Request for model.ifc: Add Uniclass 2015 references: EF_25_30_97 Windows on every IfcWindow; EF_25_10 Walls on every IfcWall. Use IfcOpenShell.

First a look at what the model holds.

```python
import ifcopenshell

model = ifcopenshell.open("model.ifc")
print(model.schema)
print("classifications:", [c.Name for c in model.by_type("IfcClassification")])
for ifc_class in ("IfcDoor", "IfcRoof", "IfcStair", "IfcWall", "IfcWindow"):
    print(ifc_class, len(model.by_type(ifc_class)))
```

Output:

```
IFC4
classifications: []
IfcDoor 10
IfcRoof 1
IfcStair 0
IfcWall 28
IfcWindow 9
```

```python
import ifcopenshell
import ifcopenshell.api.classification

model = ifcopenshell.open("model.ifc")

system = ifcopenshell.api.classification.add_classification(model, classification="Uniclass 2015")

codes = {
    "IfcWindow": ("EF_25_30_97", "Windows"),
    "IfcWall": ("EF_25_10", "Walls"),
}
for ifc_class, (code, name) in codes.items():
    products = model.by_type(ifc_class)
    ifcopenshell.api.classification.add_reference(
        model, products=products, classification=system, identification=code, name=name
    )
    print(code, len(products))

model.write("model_updated.ifc")
```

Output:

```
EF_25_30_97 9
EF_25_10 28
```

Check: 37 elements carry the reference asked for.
